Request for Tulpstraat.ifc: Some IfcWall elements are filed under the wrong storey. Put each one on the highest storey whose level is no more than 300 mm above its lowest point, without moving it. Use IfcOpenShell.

First a look at what the model holds.

```python
import ifcopenshell
import ifcopenshell.util.element
import ifcopenshell.util.placement

model = ifcopenshell.open("Tulpstraat.ifc")
print(model.schema)
for storey in model.by_type("IfcBuildingStorey"):
    level = ifcopenshell.util.placement.get_storey_elevation(storey)
    count = sum(e.is_a("IfcWall") for e in ifcopenshell.util.element.get_contained(storey))
    print(storey.id(), storey.Name, round(level, 3), count, sep=" | ")
```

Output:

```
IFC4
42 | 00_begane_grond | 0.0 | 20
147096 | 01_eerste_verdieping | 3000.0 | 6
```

```python
import ifcopenshell
import ifcopenshell.api.spatial
import ifcopenshell.geom
import ifcopenshell.util.element
import ifcopenshell.util.placement
import ifcopenshell.util.shape
import ifcopenshell.util.unit

model = ifcopenshell.open("Tulpstraat.ifc")
unit_scale = ifcopenshell.util.unit.calculate_unit_scale(model)
settings = ifcopenshell.geom.settings()

levels = sorted(
    ((ifcopenshell.util.placement.get_storey_elevation(s) * unit_scale, s) for s in model.by_type("IfcBuildingStorey")),
    key=lambda pair: pair[0],
)

for e in model.by_type("IfcWall"):
    current = e.ContainedInStructure[0].RelatingStructure if e.ContainedInStructure else None
    if current is None or not current.is_a("IfcBuildingStorey"):
        continue
    shape = ifcopenshell.geom.create_shape(settings, e)
    bottom = ifcopenshell.util.shape.get_shape_bottom_elevation(shape, shape.geometry)
    below = [s for level, s in levels if level <= bottom + 0.3]
    storey = below[-1] if below else levels[0][1]
    if storey != current:
        # assign_container keeps the world position.
        ifcopenshell.api.spatial.assign_container(model, products=[e], relating_structure=storey)
        print(e.id(), current.Name, "->", storey.Name)

model.write("Tulpstraat_edited.ifc")
```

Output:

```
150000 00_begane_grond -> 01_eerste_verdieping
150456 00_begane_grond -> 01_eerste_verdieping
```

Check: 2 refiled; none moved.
